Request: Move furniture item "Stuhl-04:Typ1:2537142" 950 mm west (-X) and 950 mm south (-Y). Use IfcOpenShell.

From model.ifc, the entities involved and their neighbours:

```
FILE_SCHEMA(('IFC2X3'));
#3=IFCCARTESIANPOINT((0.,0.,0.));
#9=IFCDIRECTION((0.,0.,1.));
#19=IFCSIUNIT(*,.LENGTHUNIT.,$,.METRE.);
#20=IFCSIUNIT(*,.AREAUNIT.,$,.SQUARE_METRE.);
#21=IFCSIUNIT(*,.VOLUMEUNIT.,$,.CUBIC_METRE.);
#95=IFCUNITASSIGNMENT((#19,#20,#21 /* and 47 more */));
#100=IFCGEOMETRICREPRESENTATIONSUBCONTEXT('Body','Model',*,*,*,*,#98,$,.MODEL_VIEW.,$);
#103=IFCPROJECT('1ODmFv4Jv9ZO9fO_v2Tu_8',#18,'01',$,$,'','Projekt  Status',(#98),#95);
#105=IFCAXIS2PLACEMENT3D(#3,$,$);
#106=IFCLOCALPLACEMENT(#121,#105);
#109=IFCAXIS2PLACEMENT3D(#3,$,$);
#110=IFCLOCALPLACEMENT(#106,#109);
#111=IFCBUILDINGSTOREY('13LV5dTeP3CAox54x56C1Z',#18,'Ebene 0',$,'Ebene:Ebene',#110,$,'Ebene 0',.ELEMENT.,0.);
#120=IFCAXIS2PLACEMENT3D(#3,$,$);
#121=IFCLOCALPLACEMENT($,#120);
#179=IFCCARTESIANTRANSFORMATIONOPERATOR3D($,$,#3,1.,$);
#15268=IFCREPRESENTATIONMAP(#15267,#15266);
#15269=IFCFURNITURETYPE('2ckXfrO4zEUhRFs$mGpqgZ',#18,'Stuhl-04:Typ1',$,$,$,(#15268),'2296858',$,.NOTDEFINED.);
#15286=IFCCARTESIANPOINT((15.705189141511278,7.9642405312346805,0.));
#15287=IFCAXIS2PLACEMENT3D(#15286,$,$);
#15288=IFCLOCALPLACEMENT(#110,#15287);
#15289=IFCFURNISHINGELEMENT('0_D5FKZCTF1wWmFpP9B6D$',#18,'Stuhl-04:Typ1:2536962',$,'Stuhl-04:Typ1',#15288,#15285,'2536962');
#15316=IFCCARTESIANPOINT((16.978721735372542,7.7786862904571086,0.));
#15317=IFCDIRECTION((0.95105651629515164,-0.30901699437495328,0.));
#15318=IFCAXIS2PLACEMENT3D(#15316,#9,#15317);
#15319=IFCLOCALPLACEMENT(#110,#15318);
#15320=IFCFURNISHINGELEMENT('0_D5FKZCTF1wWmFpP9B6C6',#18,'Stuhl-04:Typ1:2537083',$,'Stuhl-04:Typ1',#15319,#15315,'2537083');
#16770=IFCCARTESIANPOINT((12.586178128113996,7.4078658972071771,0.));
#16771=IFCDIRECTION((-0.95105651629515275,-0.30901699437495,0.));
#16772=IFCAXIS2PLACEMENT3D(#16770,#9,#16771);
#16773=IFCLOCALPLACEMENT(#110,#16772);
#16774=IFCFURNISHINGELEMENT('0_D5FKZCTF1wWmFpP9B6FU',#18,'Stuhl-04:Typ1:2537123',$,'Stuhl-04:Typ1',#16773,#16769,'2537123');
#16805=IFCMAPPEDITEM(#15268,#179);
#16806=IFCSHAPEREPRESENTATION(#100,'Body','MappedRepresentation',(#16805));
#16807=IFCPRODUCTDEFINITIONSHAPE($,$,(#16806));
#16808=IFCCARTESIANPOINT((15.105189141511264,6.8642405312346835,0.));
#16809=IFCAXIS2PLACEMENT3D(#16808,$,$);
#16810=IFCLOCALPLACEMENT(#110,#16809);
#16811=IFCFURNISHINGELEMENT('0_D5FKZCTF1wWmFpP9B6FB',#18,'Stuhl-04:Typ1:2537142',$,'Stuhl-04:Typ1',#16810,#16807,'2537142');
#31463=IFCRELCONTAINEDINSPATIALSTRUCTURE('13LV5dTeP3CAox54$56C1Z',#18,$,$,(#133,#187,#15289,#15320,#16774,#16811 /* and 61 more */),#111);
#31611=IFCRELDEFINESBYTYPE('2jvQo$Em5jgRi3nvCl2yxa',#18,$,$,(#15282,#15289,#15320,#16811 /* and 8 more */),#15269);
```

```python
import ifcopenshell
import ifcopenshell.api.geometry
import ifcopenshell.util.placement

model = ifcopenshell.open("model.ifc")

item = model.by_guid("0_D5FKZCTF1wWmFpP9B6FB")
matrix = ifcopenshell.util.placement.get_local_placement(item.ObjectPlacement)
matrix[0, 3] -= 0.95
matrix[1, 3] -= 0.95
ifcopenshell.api.geometry.edit_object_placement(model, product=item, matrix=matrix, is_si=False)

print(ifcopenshell.util.placement.get_local_placement(item.ObjectPlacement).round(3) + 0.0)

model.write("model_rev.ifc")
```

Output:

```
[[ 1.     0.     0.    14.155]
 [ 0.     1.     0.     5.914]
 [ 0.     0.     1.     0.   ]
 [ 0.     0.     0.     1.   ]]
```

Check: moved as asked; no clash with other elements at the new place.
